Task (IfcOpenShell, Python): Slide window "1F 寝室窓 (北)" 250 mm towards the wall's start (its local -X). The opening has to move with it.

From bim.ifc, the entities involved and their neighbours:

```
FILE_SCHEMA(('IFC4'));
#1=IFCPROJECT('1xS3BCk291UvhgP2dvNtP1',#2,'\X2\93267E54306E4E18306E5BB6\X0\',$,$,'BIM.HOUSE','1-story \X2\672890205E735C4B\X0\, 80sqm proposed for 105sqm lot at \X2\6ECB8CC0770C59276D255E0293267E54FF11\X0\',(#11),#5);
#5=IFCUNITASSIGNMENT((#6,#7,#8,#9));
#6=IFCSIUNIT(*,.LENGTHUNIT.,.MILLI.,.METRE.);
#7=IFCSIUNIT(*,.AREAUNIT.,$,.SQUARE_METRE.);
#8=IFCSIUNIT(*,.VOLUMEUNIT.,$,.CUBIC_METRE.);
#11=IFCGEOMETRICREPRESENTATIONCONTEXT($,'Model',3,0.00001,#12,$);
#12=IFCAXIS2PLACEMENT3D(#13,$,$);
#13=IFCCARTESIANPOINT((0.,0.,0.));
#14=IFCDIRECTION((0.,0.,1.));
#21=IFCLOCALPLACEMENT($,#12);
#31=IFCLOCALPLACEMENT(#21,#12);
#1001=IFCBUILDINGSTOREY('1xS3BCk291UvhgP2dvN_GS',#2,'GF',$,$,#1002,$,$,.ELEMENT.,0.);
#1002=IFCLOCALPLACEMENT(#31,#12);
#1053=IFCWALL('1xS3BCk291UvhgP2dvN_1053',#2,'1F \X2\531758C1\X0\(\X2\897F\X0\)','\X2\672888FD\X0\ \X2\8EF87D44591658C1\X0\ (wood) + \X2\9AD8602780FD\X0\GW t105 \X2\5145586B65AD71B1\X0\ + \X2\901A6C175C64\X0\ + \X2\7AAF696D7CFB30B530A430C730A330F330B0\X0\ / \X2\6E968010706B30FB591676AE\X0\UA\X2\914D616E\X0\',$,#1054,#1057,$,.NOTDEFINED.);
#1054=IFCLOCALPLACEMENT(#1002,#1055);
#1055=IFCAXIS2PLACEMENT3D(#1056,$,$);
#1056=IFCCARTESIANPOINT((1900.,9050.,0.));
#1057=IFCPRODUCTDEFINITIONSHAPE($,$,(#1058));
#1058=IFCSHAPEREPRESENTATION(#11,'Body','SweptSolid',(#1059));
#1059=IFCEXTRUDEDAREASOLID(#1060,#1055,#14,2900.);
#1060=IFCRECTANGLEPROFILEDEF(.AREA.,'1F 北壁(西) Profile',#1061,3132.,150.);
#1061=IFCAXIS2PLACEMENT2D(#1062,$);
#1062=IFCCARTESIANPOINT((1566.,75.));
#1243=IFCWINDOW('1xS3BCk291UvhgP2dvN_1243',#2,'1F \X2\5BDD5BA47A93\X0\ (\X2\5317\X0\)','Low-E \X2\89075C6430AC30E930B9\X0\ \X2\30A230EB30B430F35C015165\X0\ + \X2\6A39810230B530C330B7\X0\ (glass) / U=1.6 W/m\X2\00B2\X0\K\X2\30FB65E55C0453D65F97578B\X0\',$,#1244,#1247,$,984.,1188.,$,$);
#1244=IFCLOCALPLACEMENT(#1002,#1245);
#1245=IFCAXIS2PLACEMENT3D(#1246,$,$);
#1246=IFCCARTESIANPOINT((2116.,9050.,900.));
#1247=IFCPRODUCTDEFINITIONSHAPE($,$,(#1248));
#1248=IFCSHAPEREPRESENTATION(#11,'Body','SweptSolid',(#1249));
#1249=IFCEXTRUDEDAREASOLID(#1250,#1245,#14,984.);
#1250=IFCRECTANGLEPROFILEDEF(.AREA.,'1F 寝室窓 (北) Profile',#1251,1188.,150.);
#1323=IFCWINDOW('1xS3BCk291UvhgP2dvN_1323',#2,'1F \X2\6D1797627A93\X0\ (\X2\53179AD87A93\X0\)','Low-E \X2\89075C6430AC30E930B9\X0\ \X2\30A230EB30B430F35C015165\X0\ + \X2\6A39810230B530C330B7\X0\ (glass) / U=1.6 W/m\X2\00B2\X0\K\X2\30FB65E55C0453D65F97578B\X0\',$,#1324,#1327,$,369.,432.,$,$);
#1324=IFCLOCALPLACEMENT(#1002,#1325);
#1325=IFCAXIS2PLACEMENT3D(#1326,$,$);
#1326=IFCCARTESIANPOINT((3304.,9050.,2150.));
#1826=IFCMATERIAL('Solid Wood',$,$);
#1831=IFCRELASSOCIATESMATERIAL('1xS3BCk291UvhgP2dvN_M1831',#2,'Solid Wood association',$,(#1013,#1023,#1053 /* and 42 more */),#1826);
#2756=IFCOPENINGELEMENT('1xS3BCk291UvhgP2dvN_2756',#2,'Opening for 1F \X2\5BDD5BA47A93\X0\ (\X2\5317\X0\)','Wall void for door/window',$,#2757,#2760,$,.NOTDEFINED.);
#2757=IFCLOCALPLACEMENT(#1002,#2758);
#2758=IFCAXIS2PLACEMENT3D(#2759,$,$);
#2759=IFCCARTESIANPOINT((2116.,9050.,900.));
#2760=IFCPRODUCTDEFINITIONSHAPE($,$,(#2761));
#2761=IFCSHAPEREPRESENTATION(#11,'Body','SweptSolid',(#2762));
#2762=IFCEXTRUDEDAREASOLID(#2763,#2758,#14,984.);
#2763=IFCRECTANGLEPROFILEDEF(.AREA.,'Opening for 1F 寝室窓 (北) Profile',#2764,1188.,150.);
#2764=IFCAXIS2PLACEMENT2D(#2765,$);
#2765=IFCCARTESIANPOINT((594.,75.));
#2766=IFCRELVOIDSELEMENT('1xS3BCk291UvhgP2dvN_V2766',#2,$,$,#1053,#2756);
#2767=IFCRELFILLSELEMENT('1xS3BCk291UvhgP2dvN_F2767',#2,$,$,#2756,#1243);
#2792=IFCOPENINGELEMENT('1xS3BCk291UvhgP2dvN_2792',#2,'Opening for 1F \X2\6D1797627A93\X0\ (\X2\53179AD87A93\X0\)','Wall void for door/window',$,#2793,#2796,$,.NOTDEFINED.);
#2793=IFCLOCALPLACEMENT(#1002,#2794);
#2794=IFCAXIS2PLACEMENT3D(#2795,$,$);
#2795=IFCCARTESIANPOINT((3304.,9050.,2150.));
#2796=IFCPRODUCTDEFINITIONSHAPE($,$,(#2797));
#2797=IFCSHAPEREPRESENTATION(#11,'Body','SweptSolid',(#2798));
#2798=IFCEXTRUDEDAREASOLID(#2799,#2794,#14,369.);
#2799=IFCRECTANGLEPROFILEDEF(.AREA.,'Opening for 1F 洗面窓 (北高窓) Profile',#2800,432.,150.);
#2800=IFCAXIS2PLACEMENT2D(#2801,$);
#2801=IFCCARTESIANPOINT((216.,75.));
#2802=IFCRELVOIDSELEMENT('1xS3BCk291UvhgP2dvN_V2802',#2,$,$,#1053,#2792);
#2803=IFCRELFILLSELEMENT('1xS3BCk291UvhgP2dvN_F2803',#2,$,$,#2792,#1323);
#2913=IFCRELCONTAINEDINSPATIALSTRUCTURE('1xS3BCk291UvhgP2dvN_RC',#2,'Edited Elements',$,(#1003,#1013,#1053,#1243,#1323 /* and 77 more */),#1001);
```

```python
import ifcopenshell
import ifcopenshell.api.geometry
import ifcopenshell.util.placement
import ifcopenshell.util.unit

model = ifcopenshell.open("bim.ifc")
unit_scale = ifcopenshell.util.unit.calculate_unit_scale(model)

window = model.by_guid("1xS3BCk291UvhgP2dvN_1243")
opening = window.FillsVoids[0].RelatingOpeningElement
wall = opening.VoidsElements[0].RelatingBuildingElement

wall_matrix = ifcopenshell.util.placement.get_local_placement(wall.ObjectPlacement)
shift = wall_matrix[:3, 0] * -0.25 / unit_scale
before = ifcopenshell.util.placement.get_local_placement(window.ObjectPlacement)[:3, 3].copy()

# The window is not placed relative to its opening, so move both.
for product in (opening, window):
    matrix = ifcopenshell.util.placement.get_local_placement(product.ObjectPlacement)
    matrix[:3, 3] += shift
    ifcopenshell.api.geometry.edit_object_placement(model, product=product, matrix=matrix, is_si=False)

after = ifcopenshell.util.placement.get_local_placement(window.ObjectPlacement)[:3, 3]
print("window moved by", (after - before).round(3) + 0.0)

model.write("bim_updated.ifc")
```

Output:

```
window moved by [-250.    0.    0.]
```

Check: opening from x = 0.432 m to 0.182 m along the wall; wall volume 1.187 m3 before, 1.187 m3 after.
